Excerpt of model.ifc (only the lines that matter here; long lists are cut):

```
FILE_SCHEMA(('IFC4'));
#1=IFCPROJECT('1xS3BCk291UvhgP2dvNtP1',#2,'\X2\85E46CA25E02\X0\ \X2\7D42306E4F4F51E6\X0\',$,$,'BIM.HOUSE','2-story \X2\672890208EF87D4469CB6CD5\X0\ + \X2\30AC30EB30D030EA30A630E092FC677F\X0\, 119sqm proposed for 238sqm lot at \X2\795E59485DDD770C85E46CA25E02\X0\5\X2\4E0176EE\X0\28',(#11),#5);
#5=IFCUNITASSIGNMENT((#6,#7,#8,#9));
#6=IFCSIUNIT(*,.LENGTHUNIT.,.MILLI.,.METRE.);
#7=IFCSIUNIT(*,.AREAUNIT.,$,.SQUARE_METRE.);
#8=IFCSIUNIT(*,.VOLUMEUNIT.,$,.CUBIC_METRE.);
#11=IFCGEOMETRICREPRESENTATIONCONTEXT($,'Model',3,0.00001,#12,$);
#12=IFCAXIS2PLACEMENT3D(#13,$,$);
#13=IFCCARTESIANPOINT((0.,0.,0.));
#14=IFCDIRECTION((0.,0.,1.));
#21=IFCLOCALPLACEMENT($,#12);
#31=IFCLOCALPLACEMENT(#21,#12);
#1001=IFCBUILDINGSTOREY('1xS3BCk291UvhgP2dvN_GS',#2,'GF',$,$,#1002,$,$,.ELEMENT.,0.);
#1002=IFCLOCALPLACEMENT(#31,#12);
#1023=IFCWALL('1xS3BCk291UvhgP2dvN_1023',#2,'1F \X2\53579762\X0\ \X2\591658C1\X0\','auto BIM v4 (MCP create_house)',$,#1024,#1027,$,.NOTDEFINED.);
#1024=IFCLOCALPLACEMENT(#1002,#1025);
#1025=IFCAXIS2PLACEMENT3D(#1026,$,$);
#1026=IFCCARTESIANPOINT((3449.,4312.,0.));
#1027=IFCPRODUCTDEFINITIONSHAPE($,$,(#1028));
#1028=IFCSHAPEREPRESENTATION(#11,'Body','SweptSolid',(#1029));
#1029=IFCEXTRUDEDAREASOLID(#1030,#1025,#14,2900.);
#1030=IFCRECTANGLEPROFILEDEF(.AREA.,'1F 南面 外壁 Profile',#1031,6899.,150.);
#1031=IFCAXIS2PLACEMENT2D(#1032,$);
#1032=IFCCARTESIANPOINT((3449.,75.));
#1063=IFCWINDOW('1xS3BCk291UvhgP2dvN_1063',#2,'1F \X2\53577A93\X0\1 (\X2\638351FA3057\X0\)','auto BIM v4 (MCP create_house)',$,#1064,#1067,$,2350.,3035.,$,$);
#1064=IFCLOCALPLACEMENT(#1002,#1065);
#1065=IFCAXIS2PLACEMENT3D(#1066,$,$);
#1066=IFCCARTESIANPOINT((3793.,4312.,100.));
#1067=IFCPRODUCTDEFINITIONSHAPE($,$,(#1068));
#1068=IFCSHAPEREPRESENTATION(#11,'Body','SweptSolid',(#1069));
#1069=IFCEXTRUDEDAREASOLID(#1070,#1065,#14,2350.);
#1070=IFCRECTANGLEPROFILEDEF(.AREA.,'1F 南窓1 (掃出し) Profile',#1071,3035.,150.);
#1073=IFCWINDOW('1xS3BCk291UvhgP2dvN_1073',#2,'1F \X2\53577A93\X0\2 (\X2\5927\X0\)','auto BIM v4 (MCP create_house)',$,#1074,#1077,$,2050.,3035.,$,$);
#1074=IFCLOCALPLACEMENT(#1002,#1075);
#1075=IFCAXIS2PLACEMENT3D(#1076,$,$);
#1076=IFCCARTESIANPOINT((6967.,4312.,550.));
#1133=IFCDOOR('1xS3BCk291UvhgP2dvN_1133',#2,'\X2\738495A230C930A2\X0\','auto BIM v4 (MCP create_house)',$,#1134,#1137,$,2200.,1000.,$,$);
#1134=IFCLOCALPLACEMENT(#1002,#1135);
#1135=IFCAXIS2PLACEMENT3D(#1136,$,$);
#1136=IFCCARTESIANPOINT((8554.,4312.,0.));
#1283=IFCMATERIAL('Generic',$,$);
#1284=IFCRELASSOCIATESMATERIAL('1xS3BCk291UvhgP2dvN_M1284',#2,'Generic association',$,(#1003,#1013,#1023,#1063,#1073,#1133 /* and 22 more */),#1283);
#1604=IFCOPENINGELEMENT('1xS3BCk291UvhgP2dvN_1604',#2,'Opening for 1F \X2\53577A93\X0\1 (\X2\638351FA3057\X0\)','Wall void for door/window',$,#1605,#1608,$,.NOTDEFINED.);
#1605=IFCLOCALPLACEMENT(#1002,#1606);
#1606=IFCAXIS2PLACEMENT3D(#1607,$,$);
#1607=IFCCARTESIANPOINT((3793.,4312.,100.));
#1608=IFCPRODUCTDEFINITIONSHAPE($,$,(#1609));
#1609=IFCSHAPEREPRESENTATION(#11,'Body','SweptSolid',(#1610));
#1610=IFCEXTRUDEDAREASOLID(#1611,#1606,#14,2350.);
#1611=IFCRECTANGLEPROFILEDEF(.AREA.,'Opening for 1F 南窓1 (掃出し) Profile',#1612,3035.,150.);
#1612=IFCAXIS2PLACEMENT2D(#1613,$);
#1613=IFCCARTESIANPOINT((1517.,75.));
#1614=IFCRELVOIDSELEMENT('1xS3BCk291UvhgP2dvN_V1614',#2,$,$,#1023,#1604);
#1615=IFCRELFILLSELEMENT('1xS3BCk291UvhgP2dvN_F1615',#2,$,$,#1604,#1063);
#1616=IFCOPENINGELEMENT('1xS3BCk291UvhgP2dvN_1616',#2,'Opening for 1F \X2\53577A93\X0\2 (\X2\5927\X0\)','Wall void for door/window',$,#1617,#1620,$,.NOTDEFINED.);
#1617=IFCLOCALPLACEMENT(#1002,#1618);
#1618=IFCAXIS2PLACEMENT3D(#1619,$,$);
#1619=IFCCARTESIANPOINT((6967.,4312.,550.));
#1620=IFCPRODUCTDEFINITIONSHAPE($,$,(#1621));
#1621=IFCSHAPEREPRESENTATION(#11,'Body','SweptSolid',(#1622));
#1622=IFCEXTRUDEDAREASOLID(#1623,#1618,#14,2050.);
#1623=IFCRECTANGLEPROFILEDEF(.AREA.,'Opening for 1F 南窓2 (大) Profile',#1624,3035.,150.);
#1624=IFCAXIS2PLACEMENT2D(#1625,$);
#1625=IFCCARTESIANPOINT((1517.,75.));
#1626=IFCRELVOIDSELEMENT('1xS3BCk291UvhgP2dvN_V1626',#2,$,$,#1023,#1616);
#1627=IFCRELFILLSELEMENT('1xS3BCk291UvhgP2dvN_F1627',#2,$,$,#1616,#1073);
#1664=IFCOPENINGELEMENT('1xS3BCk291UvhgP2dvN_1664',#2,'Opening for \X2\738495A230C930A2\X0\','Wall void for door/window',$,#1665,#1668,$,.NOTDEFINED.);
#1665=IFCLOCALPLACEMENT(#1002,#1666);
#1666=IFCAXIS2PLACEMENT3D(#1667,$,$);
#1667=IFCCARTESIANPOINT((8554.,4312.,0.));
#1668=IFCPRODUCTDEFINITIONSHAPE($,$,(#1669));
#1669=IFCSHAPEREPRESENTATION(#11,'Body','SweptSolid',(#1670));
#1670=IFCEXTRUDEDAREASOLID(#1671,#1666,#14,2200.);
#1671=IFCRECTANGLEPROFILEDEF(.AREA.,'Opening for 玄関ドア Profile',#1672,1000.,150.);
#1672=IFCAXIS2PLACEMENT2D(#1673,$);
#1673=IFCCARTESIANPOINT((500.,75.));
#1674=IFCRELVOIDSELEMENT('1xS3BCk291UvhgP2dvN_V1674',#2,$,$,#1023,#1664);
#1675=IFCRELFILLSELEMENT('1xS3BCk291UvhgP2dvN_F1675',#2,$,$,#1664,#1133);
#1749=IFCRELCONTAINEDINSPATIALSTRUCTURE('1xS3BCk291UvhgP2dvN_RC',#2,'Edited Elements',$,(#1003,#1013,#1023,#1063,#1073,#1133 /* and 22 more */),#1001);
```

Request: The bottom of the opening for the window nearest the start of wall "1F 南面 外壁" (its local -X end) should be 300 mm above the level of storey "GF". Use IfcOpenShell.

```python
import numpy as np
import ifcopenshell
import ifcopenshell.api.geometry
import ifcopenshell.geom
import ifcopenshell.util.element
import ifcopenshell.util.placement
import ifcopenshell.util.shape
import ifcopenshell.util.unit

model = ifcopenshell.open("model.ifc")
unit_scale = ifcopenshell.util.unit.calculate_unit_scale(model)

window = model.by_id(1063)
opening = window.FillsVoids[0].RelatingOpeningElement
storey = ifcopenshell.util.element.get_container(window, ifc_class="IfcBuildingStorey")
level = ifcopenshell.util.placement.get_local_placement(storey.ObjectPlacement)[2, 3]

# The opening's origin need not be at the sill, so measure its lowest point.
shape = ifcopenshell.geom.create_shape(ifcopenshell.geom.settings(), opening)
bottom = ifcopenshell.util.shape.get_shape_bottom_elevation(shape, shape.geometry) / unit_scale
dz = level + 300.0 - bottom

shift = np.array([0.0, 0.0, dz])
# The window is not placed relative to its opening, so move both.
for product in (opening, window):
    matrix = ifcopenshell.util.placement.get_local_placement(product.ObjectPlacement)
    matrix[:3, 3] += shift
    ifcopenshell.api.geometry.edit_object_placement(model, product=product, matrix=matrix, is_si=False)

print(f"moved by {dz * unit_scale:+.3f} m")

model.write("model_updated.ifc")
```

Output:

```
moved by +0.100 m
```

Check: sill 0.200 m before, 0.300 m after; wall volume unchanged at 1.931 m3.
